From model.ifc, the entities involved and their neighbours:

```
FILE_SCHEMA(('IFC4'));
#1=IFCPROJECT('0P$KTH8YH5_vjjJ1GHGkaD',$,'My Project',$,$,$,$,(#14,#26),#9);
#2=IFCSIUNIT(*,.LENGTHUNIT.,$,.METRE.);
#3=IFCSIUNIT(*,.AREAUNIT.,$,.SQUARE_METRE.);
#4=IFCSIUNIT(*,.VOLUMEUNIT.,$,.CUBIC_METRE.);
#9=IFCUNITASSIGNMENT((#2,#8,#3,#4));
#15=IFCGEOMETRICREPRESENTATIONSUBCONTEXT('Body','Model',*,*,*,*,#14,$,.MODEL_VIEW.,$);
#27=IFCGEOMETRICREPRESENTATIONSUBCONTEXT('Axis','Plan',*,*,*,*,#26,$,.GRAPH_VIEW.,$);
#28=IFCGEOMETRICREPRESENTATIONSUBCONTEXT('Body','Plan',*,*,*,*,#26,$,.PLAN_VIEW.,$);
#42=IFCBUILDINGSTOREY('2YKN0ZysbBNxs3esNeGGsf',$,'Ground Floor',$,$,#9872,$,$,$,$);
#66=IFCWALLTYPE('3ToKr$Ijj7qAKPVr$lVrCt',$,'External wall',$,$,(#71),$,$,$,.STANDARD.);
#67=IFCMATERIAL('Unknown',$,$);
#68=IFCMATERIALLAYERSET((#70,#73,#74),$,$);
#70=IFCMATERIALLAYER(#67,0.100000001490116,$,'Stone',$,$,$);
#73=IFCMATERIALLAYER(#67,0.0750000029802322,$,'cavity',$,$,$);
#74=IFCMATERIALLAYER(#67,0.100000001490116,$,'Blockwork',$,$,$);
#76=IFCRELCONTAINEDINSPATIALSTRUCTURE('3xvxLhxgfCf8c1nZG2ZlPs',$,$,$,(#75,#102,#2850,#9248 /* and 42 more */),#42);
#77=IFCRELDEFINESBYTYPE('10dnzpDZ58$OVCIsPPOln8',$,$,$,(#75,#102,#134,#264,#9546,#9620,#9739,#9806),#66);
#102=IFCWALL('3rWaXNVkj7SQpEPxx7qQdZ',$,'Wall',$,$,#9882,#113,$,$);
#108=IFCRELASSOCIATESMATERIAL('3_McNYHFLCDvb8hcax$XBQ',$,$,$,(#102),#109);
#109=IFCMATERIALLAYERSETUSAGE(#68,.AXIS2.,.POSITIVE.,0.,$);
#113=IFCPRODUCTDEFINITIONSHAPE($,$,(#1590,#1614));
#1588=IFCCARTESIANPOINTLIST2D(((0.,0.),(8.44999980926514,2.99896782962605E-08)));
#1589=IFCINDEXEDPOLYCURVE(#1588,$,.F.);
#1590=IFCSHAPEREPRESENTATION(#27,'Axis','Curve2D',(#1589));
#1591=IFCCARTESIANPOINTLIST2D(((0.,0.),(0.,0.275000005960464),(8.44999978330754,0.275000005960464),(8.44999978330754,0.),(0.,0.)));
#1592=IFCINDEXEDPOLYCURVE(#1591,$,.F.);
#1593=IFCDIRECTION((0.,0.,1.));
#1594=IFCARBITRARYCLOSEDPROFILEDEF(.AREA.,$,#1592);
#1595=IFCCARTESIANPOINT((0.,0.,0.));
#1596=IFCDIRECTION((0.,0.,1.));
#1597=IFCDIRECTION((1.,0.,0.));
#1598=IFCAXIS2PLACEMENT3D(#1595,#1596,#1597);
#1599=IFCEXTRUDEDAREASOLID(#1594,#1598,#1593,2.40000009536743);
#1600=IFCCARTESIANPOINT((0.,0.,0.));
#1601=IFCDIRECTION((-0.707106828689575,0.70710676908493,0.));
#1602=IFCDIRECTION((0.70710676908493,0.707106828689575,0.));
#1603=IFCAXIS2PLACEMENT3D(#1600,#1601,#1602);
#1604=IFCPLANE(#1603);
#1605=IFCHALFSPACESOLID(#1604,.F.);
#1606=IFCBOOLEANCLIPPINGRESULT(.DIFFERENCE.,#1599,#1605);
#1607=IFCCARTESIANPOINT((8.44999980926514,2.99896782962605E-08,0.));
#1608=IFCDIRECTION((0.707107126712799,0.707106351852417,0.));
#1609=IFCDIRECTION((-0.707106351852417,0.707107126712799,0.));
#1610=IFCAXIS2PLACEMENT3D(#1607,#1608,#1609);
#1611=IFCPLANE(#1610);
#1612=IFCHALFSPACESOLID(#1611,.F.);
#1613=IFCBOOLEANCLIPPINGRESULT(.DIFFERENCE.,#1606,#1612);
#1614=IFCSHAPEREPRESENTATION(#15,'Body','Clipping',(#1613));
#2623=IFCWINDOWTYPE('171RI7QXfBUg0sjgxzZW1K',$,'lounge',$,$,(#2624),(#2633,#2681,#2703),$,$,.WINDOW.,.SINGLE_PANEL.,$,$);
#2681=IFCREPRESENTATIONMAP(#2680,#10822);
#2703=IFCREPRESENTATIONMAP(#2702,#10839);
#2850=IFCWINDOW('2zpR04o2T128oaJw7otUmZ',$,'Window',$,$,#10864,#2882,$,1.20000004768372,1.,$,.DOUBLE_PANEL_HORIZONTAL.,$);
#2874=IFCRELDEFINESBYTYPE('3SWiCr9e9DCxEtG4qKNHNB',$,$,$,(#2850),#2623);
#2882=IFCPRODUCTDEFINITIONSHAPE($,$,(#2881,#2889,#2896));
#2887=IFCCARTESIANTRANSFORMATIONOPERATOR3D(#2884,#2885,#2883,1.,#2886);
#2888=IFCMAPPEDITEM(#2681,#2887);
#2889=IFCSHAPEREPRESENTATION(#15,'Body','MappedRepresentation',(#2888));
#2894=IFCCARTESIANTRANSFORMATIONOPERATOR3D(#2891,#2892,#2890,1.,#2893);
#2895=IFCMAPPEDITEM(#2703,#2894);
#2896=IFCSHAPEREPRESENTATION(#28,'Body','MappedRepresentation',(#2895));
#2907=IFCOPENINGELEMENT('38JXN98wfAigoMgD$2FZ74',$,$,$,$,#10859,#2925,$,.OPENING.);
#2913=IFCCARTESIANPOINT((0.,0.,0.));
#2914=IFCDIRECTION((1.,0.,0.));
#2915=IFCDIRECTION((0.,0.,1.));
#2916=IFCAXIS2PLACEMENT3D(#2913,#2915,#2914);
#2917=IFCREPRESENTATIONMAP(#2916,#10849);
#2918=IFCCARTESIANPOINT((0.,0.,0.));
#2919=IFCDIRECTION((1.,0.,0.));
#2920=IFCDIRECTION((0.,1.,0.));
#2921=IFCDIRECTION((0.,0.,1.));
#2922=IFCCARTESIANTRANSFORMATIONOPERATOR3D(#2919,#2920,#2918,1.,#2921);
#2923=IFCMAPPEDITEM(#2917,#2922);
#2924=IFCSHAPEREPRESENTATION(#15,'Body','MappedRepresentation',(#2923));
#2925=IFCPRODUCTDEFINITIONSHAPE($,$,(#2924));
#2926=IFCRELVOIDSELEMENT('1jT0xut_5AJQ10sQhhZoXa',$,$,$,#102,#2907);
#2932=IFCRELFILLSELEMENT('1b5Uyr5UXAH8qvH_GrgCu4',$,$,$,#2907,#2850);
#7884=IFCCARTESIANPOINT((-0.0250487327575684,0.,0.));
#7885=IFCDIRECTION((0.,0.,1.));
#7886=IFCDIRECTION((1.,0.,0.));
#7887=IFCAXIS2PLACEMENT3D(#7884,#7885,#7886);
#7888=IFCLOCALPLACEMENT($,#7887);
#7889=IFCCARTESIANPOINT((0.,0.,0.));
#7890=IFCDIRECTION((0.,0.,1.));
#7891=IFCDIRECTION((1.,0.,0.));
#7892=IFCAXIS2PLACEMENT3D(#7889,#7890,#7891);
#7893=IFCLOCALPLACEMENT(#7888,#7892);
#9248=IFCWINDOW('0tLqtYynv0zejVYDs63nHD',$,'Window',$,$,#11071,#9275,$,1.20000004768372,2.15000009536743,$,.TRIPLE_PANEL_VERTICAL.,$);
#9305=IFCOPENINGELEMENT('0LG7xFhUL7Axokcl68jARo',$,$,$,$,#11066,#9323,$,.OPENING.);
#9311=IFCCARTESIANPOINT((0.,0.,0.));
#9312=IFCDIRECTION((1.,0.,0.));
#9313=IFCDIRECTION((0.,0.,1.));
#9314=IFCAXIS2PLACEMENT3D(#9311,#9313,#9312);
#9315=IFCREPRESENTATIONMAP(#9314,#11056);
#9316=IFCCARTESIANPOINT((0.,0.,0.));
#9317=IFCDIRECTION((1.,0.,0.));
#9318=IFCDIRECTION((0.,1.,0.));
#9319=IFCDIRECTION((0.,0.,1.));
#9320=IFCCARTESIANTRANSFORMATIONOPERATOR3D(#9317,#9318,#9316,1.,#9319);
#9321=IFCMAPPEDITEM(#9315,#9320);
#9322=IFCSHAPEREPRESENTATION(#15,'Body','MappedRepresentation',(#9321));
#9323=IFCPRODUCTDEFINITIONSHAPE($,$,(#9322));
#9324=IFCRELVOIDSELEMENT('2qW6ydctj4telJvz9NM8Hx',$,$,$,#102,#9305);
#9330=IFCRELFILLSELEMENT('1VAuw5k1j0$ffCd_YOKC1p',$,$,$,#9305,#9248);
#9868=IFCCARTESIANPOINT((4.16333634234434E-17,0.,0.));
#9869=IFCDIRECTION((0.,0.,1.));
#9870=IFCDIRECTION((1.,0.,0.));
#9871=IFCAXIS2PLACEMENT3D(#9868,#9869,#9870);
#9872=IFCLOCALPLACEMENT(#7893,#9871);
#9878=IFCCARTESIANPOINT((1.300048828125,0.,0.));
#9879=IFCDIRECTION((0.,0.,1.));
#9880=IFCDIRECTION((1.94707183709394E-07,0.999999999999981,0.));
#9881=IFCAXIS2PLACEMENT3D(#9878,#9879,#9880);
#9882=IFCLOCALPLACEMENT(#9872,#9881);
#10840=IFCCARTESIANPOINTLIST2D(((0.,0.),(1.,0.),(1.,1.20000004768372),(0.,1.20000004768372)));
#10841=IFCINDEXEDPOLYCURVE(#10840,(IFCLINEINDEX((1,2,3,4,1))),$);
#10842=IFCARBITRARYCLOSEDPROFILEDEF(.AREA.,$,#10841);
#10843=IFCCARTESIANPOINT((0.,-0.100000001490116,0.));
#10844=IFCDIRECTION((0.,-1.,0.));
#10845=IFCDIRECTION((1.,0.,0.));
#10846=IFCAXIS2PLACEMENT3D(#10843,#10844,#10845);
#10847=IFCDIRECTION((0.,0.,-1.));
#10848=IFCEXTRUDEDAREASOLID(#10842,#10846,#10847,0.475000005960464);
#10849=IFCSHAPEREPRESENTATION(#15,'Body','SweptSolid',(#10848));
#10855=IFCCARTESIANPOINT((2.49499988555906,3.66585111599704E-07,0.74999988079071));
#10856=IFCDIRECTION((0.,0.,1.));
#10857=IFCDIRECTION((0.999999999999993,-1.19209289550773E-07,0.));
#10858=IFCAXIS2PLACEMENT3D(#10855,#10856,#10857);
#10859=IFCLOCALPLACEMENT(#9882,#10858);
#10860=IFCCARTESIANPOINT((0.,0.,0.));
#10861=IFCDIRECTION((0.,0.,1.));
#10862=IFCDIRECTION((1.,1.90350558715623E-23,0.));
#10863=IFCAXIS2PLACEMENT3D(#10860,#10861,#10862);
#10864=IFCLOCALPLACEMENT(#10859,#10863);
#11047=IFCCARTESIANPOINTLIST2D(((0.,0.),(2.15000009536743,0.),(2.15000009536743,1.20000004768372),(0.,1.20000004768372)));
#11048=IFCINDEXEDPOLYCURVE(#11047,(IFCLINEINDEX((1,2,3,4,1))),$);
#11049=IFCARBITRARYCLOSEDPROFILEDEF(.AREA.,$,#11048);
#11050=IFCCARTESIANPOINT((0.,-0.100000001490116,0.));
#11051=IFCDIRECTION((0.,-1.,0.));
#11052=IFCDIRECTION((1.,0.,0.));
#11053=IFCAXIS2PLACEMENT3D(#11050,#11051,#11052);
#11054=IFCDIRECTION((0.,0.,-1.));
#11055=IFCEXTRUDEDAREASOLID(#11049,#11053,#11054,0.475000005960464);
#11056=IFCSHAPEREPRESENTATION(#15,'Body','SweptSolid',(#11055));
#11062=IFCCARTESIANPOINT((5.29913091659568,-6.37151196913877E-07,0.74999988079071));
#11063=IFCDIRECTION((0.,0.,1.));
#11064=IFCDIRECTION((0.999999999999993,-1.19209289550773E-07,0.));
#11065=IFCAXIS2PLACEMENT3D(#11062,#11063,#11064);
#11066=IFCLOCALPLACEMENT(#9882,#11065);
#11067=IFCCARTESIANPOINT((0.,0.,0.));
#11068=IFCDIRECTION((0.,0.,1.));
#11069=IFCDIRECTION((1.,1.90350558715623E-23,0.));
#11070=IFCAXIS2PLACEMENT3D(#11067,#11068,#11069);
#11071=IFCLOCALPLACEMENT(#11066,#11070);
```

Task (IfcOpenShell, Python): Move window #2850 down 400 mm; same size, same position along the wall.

```python
import numpy as np
import ifcopenshell
import ifcopenshell.api.geometry
import ifcopenshell.util.placement
import ifcopenshell.util.unit

model = ifcopenshell.open("model.ifc")
unit_scale = ifcopenshell.util.unit.calculate_unit_scale(model)

window = model.by_id(2850)
opening = window.FillsVoids[0].RelatingOpeningElement
dz = -0.4 / unit_scale

shift = np.array([0.0, 0.0, dz])
# The window is placed relative to its opening, so it follows when the opening moves.
matrix = ifcopenshell.util.placement.get_local_placement(opening.ObjectPlacement)
matrix[:3, 3] += shift
ifcopenshell.api.geometry.edit_object_placement(
    model, product=opening, matrix=matrix, is_si=False, should_transform_children=True
)

print(f"moved by {dz * unit_scale:+.3f} m")

model.write("model_rev.ifc")
```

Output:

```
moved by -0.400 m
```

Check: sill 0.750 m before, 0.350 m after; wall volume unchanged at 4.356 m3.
